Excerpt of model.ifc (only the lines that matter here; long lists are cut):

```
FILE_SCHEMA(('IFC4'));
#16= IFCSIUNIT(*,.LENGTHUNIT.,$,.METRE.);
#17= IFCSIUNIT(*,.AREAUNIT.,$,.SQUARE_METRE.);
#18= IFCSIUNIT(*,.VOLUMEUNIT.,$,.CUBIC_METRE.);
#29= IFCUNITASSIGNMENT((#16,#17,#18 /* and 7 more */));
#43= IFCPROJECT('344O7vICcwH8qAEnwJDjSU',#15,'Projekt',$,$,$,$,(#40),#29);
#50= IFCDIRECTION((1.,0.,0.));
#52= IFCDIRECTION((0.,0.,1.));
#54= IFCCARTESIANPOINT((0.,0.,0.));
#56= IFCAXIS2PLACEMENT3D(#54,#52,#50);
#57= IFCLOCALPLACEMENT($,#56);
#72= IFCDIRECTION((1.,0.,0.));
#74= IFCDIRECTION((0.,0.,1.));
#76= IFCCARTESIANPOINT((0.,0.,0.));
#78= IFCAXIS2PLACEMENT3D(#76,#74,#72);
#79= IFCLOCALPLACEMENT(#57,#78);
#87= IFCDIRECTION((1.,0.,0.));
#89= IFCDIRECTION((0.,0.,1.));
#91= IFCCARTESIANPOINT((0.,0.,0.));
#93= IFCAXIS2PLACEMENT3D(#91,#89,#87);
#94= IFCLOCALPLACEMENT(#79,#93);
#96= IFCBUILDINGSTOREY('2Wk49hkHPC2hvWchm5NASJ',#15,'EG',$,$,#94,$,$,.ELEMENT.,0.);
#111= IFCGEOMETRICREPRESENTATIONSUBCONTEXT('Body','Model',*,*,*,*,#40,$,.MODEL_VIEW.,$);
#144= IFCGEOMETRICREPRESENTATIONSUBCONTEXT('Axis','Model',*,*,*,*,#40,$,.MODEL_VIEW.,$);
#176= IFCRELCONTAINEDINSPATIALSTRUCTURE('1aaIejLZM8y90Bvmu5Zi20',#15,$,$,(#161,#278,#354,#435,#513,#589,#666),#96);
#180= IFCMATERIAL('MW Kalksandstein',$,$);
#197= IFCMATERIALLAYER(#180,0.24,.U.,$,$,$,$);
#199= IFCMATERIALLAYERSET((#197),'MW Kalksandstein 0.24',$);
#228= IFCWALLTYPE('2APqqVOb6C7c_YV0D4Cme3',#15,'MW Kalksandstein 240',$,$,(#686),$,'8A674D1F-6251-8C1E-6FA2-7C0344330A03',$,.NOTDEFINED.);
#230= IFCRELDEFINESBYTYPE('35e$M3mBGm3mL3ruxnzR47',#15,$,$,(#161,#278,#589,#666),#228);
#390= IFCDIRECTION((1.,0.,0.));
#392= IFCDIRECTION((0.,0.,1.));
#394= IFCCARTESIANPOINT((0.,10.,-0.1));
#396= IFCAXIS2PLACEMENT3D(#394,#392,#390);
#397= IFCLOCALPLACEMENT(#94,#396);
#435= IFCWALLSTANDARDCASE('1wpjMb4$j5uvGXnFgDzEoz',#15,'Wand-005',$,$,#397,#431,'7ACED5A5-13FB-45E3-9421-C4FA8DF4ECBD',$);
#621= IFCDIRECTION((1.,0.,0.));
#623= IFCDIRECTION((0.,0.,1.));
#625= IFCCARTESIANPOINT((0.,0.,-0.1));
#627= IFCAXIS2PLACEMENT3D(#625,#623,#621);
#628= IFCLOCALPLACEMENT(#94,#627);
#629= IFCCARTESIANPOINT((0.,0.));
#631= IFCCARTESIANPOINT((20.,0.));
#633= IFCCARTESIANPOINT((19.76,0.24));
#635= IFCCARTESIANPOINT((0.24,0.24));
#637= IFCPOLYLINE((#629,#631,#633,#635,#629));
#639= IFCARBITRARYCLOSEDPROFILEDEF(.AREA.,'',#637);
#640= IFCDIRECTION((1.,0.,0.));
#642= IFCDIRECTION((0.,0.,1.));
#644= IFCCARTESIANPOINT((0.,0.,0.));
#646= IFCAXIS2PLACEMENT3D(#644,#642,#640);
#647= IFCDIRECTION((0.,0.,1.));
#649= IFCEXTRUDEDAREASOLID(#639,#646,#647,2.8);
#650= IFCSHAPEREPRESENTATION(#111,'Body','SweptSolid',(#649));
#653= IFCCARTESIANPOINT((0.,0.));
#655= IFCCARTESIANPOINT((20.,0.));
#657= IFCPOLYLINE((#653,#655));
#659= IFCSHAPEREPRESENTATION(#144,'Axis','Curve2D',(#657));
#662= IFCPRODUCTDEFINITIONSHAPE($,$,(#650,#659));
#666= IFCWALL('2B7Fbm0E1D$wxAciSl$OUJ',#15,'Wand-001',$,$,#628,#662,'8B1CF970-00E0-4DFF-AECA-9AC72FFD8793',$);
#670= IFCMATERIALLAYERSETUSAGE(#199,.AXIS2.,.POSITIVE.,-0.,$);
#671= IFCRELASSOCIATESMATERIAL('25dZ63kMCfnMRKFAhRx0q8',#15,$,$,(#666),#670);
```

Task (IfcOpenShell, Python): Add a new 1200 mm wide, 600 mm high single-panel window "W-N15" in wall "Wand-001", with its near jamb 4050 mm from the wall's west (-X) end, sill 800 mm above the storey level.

```python
import numpy as np
import ifcopenshell
import ifcopenshell.api.feature
import ifcopenshell.api.geometry
import ifcopenshell.api.root
import ifcopenshell.api.spatial
import ifcopenshell.geom
import ifcopenshell.util.element
import ifcopenshell.util.placement
import ifcopenshell.util.representation
import ifcopenshell.util.shape
import ifcopenshell.util.unit

model = ifcopenshell.open("model.ifc")
unit_scale = ifcopenshell.util.unit.calculate_unit_scale(model)
settings = ifcopenshell.geom.settings()


def volume(element):
    """Net volume in cubic metres, openings subtracted."""
    shape = ifcopenshell.geom.create_shape(settings, element)
    return ifcopenshell.util.shape.get_volume(shape.geometry)


wall = model.by_guid("2B7Fbm0E1D$wxAciSl$OUJ")
storey = ifcopenshell.util.element.get_container(wall, ifc_class="IfcBuildingStorey")
context = ifcopenshell.util.representation.get_context(model, "Model", "Body", "MODEL_VIEW")
before = volume(wall)

width, height, from_end, sill = 1.2, 0.6, 4.05, 0.8  # metres

# The wall runs along its own X axis, and the end named is its -X end.
wall_shape = ifcopenshell.geom.create_shape(settings, wall)
x, y, z = ifcopenshell.util.shape.get_vertices(wall_shape.geometry).T
start = x.min() + from_end
face, thickness = float(y.min()), float(y.max() - y.min())
wall_matrix = ifcopenshell.util.placement.get_local_placement(wall.ObjectPlacement)
level = ifcopenshell.util.placement.get_local_placement(storey.ObjectPlacement)[2, 3]


def in_wall(x, y):
    """Placement at x, y metres in the wall's axes, at sill height."""
    matrix = wall_matrix.copy()
    matrix[:, 3] = wall_matrix @ np.array([x / unit_scale, y / unit_scale, 0.0, 1.0])
    matrix[2, 3] = level + sill / unit_scale
    return matrix


# Opening: a box that overshoots both wall faces by 50 mm.
opening = ifcopenshell.api.root.create_entity(model, ifc_class="IfcOpeningElement", predefined_type="OPENING")
box = ifcopenshell.api.geometry.add_wall_representation(
    model, context=context, length=width, height=height, thickness=thickness + 0.1
)
ifcopenshell.api.geometry.assign_representation(model, product=opening, representation=box)
ifcopenshell.api.geometry.edit_object_placement(model, product=opening, matrix=in_wall(start, face - 0.05), is_si=False)
ifcopenshell.api.feature.add_feature(model, feature=opening, element=wall)

window = ifcopenshell.api.root.create_entity(model, ifc_class="IfcWindow", name="W-N15", predefined_type="WINDOW")
window.OverallWidth, window.OverallHeight = width / unit_scale, height / unit_scale
window.PartitioningType = "SINGLE_PANEL"
body = ifcopenshell.api.geometry.add_window_representation(
    model,
    context=context,
    overall_width=window.OverallWidth,
    overall_height=window.OverallHeight,
    partition_type="SINGLE_PANEL",
)
ifcopenshell.api.geometry.assign_representation(model, product=window, representation=body)
ifcopenshell.api.spatial.assign_container(model, products=[window], relating_structure=storey)
ifcopenshell.api.feature.add_filling(model, opening=opening, element=window)

# Centre the window in the wall's thickness.
ifcopenshell.api.geometry.edit_object_placement(model, product=window, matrix=in_wall(start, face), is_si=False)
window_shape = ifcopenshell.geom.create_shape(settings, window)
depth = ifcopenshell.util.shape.get_vertices(window_shape.geometry)[:, 1]
offset = face + thickness / 2 - (depth.min() + depth.max()) / 2
ifcopenshell.api.geometry.edit_object_placement(model, product=window, matrix=in_wall(start, offset), is_si=False)

after = volume(wall)

print(f"wall volume {before:.3f} -> {after:.3f} m3")

model.write("model_rev.ifc")
```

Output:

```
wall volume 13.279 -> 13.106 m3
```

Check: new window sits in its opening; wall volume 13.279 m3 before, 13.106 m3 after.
